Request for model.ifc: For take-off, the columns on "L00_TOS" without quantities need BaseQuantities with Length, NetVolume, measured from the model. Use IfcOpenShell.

First a look at what the model holds.

```python
import ifcopenshell
import ifcopenshell.util.element
import ifcopenshell.util.unit

model = ifcopenshell.open("model.ifc")
print(model.schema)
for unit_type in ("LENGTHUNIT", "AREAUNIT", "VOLUMEUNIT"):
    print(unit_type, ifcopenshell.util.unit.calculate_unit_scale(model, unit_type))
storey = next(s for s in model.by_type("IfcBuildingStorey") if s.Name == "L00_TOS")
columns = [e for e in ifcopenshell.util.element.get_decomposition(storey) if e.is_a("IfcColumn")]
for e in sorted(columns, key=lambda e: e.id()):
    print(e.id(), e.is_a(), e.Name, list(ifcopenshell.util.element.get_psets(e, qtos_only=True)), sep=" | ")
```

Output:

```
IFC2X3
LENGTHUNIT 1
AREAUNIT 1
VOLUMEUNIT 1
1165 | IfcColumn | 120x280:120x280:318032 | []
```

```python
import ifcopenshell
import ifcopenshell.api.pset
import ifcopenshell.geom
import ifcopenshell.util.element
import ifcopenshell.util.shape
import ifcopenshell.util.unit

model = ifcopenshell.open("model.ifc")
unit_scale = ifcopenshell.util.unit.calculate_unit_scale(model)
volume_scale = ifcopenshell.util.unit.calculate_unit_scale(model, "VOLUMEUNIT")
settings = ifcopenshell.geom.settings()

storey = next(s for s in model.by_type("IfcBuildingStorey") if s.Name == "L00_TOS")
columns = [e for e in ifcopenshell.util.element.get_decomposition(storey) if e.is_a("IfcColumn")]

for e in sorted(columns, key=lambda e: e.id()):
    if ifcopenshell.util.element.get_psets(e, qtos_only=True, should_inherit=False):
        continue
    # Geometry comes back in metres, in the element's own axes.
    shape = ifcopenshell.geom.create_shape(settings, e)
    values = {
        "Length": ifcopenshell.util.shape.get_z(shape.geometry) / unit_scale,
        "NetVolume": ifcopenshell.util.shape.get_volume(shape.geometry) / volume_scale,
    }
    qto = ifcopenshell.api.pset.add_qto(model, product=e, name="BaseQuantities")
    ifcopenshell.api.pset.edit_qto(model, qto=qto, properties=values)
    print(e.id(), {k: round(v, 3) for k, v in values.items()})

model.write("model_v2.ifc")
```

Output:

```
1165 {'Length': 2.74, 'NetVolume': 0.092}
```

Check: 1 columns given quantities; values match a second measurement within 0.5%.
